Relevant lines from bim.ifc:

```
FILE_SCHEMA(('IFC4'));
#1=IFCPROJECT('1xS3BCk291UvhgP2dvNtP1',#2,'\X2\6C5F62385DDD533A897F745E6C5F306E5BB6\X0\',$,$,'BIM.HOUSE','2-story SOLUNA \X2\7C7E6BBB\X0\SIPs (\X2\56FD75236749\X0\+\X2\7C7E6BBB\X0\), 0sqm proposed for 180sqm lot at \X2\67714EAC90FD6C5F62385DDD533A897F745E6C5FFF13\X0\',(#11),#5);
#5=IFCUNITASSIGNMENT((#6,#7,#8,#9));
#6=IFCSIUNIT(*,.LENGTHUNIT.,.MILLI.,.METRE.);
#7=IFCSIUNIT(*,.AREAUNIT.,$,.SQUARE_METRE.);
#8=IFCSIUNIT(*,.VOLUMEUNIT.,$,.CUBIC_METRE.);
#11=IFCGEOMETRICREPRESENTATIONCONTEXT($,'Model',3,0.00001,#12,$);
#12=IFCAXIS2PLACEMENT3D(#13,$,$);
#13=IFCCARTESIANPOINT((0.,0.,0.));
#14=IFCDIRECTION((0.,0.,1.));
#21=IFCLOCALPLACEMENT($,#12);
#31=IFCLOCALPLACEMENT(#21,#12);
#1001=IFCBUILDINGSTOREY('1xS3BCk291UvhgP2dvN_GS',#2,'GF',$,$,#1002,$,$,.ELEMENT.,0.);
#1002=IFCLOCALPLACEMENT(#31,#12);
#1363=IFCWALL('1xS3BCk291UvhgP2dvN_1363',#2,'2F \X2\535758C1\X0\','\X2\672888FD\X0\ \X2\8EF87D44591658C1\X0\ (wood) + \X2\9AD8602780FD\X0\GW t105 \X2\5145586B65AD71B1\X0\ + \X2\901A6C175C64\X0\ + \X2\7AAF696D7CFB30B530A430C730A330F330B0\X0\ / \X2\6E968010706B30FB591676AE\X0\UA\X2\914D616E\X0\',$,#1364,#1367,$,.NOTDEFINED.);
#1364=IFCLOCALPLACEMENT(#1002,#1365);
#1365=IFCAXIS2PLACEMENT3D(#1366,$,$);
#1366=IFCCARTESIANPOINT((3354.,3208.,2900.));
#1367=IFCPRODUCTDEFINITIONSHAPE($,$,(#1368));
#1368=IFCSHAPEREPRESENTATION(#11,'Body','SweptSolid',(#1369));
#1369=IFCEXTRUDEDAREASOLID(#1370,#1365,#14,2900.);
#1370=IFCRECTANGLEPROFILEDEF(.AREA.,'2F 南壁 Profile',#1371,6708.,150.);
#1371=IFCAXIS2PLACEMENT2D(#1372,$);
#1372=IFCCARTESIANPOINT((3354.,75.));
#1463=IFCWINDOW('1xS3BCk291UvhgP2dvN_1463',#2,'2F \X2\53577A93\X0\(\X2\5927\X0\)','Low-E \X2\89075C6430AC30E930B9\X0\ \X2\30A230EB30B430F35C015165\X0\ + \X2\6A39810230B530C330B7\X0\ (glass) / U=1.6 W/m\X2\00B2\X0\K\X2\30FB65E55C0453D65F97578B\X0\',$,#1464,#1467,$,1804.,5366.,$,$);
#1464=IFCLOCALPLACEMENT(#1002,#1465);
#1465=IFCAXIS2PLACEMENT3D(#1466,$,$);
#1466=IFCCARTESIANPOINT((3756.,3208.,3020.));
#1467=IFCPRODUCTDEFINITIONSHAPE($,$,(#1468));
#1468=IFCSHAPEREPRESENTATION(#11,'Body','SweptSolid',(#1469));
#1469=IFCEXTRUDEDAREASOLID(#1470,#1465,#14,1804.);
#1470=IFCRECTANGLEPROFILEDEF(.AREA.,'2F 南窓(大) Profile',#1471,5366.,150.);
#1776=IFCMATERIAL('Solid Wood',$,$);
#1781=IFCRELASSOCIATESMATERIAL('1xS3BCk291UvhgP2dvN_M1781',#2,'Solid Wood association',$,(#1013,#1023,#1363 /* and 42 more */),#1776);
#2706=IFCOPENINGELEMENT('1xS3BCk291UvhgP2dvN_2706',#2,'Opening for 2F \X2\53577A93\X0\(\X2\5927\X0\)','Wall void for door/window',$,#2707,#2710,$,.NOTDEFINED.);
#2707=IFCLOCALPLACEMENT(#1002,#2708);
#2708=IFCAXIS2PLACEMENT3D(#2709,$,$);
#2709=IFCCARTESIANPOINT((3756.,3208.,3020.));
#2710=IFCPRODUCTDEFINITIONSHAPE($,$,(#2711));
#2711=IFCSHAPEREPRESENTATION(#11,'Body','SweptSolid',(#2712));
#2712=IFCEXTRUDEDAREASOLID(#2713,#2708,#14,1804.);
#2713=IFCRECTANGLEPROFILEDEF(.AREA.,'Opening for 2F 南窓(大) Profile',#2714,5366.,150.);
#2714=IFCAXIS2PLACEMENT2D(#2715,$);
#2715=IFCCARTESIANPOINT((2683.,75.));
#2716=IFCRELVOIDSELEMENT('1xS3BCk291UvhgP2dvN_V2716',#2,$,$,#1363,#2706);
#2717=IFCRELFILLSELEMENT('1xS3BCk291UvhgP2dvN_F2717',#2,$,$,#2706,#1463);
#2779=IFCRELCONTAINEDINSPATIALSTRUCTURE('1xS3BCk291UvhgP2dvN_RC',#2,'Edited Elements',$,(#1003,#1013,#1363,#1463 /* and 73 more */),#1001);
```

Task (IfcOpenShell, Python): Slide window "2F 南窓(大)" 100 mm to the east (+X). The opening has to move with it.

```python
import ifcopenshell
import ifcopenshell.api.geometry
import ifcopenshell.util.placement
import ifcopenshell.util.unit

model = ifcopenshell.open("bim.ifc")
unit_scale = ifcopenshell.util.unit.calculate_unit_scale(model)

window = model.by_id(1463)
opening = window.FillsVoids[0].RelatingOpeningElement
wall = opening.VoidsElements[0].RelatingBuildingElement

wall_matrix = ifcopenshell.util.placement.get_local_placement(wall.ObjectPlacement)
shift = wall_matrix[:3, 0] * 0.1 / unit_scale
before = ifcopenshell.util.placement.get_local_placement(window.ObjectPlacement)[:3, 3].copy()

# The window is not placed relative to its opening, so move both.
for product in (opening, window):
    matrix = ifcopenshell.util.placement.get_local_placement(product.ObjectPlacement)
    matrix[:3, 3] += shift
    ifcopenshell.api.geometry.edit_object_placement(model, product=product, matrix=matrix, is_si=False)

after = ifcopenshell.util.placement.get_local_placement(window.ObjectPlacement)[:3, 3]
print("window moved by", (after - before).round(3) + 0.0)

model.write("bim_v2.ifc")
```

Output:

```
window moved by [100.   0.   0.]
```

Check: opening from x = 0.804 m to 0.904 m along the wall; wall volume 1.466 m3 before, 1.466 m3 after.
